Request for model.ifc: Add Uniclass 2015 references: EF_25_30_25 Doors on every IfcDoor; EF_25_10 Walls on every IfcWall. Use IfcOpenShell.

First a look at what the model holds.

```python
import ifcopenshell

model = ifcopenshell.open("model.ifc")
print(model.schema)
print("classifications:", [c.Name for c in model.by_type("IfcClassification")])
for ifc_class in ("IfcDoor", "IfcRoof", "IfcStair", "IfcWall", "IfcWindow"):
    print(ifc_class, len(model.by_type(ifc_class)))
```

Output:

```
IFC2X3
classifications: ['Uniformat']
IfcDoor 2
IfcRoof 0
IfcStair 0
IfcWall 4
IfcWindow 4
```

```python
import ifcopenshell
import ifcopenshell.api.classification

model = ifcopenshell.open("model.ifc")

# IFC2X3 requires Source and Edition and has no link from the project to the system.
system = model.create_entity("IfcClassification", Source="NBS", Edition="2015", Name="Uniclass 2015")

codes = {
    "IfcDoor": ("EF_25_30_25", "Doors"),
    "IfcWall": ("EF_25_10", "Walls"),
}
for ifc_class, (code, name) in codes.items():
    products = model.by_type(ifc_class)
    ifcopenshell.api.classification.add_reference(
        model, products=products, classification=system, identification=code, name=name
    )
    print(code, len(products))

model.write("model_edited.ifc")
```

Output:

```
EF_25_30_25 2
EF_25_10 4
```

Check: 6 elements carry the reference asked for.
